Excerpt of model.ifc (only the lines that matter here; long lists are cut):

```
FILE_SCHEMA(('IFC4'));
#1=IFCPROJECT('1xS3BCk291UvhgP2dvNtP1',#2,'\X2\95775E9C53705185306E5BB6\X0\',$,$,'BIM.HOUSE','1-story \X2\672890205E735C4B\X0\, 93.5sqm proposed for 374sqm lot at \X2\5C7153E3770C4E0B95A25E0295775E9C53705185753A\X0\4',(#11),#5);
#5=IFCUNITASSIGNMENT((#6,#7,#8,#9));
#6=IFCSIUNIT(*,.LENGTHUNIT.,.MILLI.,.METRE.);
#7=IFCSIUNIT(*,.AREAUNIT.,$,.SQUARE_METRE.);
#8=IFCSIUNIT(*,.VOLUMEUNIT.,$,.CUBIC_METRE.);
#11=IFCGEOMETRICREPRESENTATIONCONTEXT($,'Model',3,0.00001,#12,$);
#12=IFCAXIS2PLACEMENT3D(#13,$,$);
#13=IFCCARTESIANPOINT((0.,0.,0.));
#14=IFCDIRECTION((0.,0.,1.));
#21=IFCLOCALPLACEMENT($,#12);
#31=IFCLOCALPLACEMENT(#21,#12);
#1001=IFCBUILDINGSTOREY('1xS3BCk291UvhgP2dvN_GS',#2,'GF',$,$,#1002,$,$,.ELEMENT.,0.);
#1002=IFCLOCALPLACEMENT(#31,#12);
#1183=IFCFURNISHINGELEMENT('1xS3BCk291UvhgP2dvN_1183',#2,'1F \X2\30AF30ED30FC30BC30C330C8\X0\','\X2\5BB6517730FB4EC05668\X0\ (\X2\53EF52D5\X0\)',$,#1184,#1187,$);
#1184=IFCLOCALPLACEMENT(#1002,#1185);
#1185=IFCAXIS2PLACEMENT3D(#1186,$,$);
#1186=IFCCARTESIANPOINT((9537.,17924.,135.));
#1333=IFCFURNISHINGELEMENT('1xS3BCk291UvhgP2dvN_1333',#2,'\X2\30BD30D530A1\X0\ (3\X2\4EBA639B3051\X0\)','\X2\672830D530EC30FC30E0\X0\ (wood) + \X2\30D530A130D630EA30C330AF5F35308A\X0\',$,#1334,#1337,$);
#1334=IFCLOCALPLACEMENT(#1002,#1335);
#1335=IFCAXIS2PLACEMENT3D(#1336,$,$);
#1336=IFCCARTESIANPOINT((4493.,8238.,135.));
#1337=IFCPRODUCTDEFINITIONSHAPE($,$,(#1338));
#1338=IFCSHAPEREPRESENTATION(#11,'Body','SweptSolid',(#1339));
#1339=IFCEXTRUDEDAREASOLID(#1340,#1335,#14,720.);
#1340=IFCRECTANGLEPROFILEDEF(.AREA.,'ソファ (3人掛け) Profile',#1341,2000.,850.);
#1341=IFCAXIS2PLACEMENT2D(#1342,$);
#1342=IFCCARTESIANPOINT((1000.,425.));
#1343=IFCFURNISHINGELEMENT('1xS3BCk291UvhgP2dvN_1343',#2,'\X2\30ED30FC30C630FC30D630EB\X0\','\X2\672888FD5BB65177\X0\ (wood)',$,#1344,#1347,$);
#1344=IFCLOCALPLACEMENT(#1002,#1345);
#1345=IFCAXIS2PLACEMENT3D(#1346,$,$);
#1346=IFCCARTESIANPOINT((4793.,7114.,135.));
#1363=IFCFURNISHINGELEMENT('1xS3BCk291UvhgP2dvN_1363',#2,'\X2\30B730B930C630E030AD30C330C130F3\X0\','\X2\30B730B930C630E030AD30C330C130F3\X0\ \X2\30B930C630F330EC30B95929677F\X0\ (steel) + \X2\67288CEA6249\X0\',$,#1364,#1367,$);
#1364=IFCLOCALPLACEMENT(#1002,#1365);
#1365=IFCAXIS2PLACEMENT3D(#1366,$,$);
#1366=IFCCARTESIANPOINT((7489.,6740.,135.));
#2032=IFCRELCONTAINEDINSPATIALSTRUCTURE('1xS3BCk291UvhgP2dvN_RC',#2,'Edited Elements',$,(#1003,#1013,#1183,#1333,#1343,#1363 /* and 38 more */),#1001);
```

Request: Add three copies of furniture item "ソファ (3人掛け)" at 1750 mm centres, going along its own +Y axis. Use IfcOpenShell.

```python
import ifcopenshell
import ifcopenshell.api.geometry
import ifcopenshell.api.root
import ifcopenshell.util.element
import ifcopenshell.util.placement
import ifcopenshell.util.unit

model = ifcopenshell.open("model.ifc")
unit_scale = ifcopenshell.util.unit.calculate_unit_scale(model)


def reuse_history(source, copy):
    """copy_class also copies each property set's owner history, people and application; keep the originals."""
    for rel in copy.IsDefinedBy:
        if rel.is_a("IfcRelDefinesByProperties") and (history := rel.RelatingPropertyDefinition.OwnerHistory):
            rel.RelatingPropertyDefinition.OwnerHistory = source.OwnerHistory
            ifcopenshell.util.element.remove_deep2(model, history)


source = model.by_guid("1xS3BCk291UvhgP2dvN_1333")
base = ifcopenshell.util.placement.get_local_placement(source.ObjectPlacement)
step = base[:3, 1] * 1.75 / unit_scale

for i in range(1, 4):
    copy = ifcopenshell.api.root.copy_class(model, product=source)
    copy.Representation = ifcopenshell.util.element.copy_deep(
        model, source.Representation, exclude=["IfcGeometricRepresentationContext", "IfcRepresentationMap"]
    )
    reuse_history(source, copy)
    matrix = base.copy()
    matrix[:3, 3] += i * step
    print("added at", matrix[:3, 3].round(3) + 0.0)
    ifcopenshell.api.geometry.edit_object_placement(model, product=copy, matrix=matrix, is_si=False)

model.write("model-out.ifc")
```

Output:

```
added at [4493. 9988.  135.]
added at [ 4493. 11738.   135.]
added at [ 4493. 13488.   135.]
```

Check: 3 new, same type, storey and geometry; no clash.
